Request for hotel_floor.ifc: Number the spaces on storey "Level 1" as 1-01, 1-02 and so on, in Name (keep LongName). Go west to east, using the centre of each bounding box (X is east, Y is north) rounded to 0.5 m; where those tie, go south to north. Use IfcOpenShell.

First a look at what the model holds.

```python
import ifcopenshell
import ifcopenshell.util.element
import ifcopenshell.util.placement

model = ifcopenshell.open("hotel_floor.ifc")
print(model.schema)
storey = next(s for s in model.by_type("IfcBuildingStorey") if s.Name == "Level 1")
spaces = [e for e in ifcopenshell.util.element.get_decomposition(storey) if e.is_a("IfcSpace")]
for e in sorted(spaces, key=lambda e: e.id()):
    origin = ifcopenshell.util.placement.get_local_placement(e.ObjectPlacement)[:3, 3]
    print(e.id(), e.Name, e.LongName, origin.round(2) + 0.0, sep=" | ")
```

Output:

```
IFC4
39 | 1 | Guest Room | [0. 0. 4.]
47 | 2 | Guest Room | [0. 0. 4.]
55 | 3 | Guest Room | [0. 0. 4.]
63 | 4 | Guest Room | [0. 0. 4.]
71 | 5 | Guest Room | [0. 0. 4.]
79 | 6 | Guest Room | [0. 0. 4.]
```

```python
import ifcopenshell
import ifcopenshell.geom
import ifcopenshell.util.element
import ifcopenshell.util.shape

model = ifcopenshell.open("hotel_floor.ifc")
settings = ifcopenshell.geom.settings()
settings.set("use-world-coords", True)


def centre(element):
    shape = ifcopenshell.geom.create_shape(settings, element)
    return ifcopenshell.util.shape.get_bbox_centroid(shape.geometry)


storey = next(s for s in model.by_type("IfcBuildingStorey") if s.Name == "Level 1")
spaces = [e for e in ifcopenshell.util.element.get_decomposition(storey) if e.is_a("IfcSpace")]

# Insertion points can sit at a corner or the storey origin, so sort by the geometry (in metres).
centres = {e: centre(e) for e in spaces}
spaces.sort(key=lambda e: (round(centres[e][0] / 0.5), centres[e][1]))

for i, e in enumerate(spaces, start=1):
    number = f"1-{i:02d}"
    e.Name = number
    print(e.id(), number)

model.write("hotel_floor_updated.ifc")
```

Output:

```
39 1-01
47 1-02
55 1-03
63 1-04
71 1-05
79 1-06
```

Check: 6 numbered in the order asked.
